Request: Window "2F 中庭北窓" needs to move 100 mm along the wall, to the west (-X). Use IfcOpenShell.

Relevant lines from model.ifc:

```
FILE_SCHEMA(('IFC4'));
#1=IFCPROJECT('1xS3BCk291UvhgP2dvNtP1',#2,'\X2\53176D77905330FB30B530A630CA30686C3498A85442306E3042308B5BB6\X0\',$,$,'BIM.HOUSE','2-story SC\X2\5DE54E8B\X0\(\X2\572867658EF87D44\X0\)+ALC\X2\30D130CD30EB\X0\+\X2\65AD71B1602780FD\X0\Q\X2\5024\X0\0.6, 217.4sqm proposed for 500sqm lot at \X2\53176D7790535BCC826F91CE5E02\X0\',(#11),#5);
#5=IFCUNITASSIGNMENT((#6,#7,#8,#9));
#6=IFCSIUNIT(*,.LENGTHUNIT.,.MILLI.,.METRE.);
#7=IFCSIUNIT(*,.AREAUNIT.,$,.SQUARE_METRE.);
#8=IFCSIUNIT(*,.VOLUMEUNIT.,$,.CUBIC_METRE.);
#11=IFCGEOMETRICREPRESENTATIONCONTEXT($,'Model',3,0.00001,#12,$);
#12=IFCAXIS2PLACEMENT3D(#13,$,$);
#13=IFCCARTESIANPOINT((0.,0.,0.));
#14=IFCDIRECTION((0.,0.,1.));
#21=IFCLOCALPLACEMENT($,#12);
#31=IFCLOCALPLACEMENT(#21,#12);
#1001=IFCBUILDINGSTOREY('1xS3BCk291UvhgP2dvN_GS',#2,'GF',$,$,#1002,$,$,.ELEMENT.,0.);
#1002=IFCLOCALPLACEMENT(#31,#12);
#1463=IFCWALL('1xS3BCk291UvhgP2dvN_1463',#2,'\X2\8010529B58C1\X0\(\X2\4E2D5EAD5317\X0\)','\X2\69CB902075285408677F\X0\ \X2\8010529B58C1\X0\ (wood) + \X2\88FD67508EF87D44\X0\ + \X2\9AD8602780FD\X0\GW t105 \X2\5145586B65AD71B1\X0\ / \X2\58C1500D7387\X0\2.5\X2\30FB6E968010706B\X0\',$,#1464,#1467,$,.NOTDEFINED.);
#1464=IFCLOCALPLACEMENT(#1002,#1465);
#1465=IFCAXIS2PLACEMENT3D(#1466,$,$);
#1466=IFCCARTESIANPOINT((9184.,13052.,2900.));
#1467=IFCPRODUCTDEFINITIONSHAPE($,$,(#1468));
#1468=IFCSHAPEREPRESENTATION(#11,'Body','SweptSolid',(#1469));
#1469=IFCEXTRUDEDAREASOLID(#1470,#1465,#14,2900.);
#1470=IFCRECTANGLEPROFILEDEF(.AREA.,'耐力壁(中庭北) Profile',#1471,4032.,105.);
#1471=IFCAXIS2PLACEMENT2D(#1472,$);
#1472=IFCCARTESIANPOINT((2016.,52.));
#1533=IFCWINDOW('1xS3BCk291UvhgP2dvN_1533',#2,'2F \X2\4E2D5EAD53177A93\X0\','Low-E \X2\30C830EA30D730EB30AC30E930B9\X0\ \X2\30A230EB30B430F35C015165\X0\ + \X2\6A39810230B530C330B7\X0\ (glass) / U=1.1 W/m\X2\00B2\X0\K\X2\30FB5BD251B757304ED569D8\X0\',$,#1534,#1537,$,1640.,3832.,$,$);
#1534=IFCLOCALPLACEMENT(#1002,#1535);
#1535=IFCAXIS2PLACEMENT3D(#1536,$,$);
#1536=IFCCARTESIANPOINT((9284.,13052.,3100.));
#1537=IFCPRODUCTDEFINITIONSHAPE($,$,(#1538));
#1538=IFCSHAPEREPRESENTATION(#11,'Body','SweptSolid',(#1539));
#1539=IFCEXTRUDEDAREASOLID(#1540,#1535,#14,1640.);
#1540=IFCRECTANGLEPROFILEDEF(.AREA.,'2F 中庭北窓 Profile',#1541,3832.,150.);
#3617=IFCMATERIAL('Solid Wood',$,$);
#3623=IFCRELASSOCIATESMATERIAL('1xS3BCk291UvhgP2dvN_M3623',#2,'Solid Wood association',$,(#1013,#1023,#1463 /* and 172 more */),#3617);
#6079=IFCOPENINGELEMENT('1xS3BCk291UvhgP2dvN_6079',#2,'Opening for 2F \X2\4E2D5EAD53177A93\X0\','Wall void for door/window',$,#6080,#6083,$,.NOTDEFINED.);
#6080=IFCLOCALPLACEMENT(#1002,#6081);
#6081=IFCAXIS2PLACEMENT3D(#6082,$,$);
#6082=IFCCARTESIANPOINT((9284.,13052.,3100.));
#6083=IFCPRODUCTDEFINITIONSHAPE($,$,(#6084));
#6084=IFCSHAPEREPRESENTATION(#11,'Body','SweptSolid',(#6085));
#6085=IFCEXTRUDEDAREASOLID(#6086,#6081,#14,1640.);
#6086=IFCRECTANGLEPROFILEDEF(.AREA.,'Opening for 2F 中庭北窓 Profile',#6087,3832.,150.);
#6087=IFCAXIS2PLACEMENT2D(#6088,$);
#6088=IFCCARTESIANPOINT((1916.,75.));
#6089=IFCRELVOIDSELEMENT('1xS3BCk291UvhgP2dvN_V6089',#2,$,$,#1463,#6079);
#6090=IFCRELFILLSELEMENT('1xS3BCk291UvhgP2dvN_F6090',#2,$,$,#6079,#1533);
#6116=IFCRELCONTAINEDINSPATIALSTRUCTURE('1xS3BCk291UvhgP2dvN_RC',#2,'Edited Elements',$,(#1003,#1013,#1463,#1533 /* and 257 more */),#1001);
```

```python
import ifcopenshell
import ifcopenshell.api.geometry
import ifcopenshell.util.placement
import ifcopenshell.util.unit

model = ifcopenshell.open("model.ifc")
unit_scale = ifcopenshell.util.unit.calculate_unit_scale(model)

window = model.by_id(1533)
opening = window.FillsVoids[0].RelatingOpeningElement
wall = opening.VoidsElements[0].RelatingBuildingElement

wall_matrix = ifcopenshell.util.placement.get_local_placement(wall.ObjectPlacement)
shift = wall_matrix[:3, 0] * -0.1 / unit_scale
before = ifcopenshell.util.placement.get_local_placement(window.ObjectPlacement)[:3, 3].copy()

# The window is not placed relative to its opening, so move both.
for product in (opening, window):
    matrix = ifcopenshell.util.placement.get_local_placement(product.ObjectPlacement)
    matrix[:3, 3] += shift
    ifcopenshell.api.geometry.edit_object_placement(model, product=product, matrix=matrix, is_si=False)

after = ifcopenshell.util.placement.get_local_placement(window.ObjectPlacement)[:3, 3]
print("window moved by", (after - before).round(3) + 0.0)

model.write("model_rev.ifc")
```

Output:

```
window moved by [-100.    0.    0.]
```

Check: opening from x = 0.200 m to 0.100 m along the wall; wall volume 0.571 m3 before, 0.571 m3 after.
